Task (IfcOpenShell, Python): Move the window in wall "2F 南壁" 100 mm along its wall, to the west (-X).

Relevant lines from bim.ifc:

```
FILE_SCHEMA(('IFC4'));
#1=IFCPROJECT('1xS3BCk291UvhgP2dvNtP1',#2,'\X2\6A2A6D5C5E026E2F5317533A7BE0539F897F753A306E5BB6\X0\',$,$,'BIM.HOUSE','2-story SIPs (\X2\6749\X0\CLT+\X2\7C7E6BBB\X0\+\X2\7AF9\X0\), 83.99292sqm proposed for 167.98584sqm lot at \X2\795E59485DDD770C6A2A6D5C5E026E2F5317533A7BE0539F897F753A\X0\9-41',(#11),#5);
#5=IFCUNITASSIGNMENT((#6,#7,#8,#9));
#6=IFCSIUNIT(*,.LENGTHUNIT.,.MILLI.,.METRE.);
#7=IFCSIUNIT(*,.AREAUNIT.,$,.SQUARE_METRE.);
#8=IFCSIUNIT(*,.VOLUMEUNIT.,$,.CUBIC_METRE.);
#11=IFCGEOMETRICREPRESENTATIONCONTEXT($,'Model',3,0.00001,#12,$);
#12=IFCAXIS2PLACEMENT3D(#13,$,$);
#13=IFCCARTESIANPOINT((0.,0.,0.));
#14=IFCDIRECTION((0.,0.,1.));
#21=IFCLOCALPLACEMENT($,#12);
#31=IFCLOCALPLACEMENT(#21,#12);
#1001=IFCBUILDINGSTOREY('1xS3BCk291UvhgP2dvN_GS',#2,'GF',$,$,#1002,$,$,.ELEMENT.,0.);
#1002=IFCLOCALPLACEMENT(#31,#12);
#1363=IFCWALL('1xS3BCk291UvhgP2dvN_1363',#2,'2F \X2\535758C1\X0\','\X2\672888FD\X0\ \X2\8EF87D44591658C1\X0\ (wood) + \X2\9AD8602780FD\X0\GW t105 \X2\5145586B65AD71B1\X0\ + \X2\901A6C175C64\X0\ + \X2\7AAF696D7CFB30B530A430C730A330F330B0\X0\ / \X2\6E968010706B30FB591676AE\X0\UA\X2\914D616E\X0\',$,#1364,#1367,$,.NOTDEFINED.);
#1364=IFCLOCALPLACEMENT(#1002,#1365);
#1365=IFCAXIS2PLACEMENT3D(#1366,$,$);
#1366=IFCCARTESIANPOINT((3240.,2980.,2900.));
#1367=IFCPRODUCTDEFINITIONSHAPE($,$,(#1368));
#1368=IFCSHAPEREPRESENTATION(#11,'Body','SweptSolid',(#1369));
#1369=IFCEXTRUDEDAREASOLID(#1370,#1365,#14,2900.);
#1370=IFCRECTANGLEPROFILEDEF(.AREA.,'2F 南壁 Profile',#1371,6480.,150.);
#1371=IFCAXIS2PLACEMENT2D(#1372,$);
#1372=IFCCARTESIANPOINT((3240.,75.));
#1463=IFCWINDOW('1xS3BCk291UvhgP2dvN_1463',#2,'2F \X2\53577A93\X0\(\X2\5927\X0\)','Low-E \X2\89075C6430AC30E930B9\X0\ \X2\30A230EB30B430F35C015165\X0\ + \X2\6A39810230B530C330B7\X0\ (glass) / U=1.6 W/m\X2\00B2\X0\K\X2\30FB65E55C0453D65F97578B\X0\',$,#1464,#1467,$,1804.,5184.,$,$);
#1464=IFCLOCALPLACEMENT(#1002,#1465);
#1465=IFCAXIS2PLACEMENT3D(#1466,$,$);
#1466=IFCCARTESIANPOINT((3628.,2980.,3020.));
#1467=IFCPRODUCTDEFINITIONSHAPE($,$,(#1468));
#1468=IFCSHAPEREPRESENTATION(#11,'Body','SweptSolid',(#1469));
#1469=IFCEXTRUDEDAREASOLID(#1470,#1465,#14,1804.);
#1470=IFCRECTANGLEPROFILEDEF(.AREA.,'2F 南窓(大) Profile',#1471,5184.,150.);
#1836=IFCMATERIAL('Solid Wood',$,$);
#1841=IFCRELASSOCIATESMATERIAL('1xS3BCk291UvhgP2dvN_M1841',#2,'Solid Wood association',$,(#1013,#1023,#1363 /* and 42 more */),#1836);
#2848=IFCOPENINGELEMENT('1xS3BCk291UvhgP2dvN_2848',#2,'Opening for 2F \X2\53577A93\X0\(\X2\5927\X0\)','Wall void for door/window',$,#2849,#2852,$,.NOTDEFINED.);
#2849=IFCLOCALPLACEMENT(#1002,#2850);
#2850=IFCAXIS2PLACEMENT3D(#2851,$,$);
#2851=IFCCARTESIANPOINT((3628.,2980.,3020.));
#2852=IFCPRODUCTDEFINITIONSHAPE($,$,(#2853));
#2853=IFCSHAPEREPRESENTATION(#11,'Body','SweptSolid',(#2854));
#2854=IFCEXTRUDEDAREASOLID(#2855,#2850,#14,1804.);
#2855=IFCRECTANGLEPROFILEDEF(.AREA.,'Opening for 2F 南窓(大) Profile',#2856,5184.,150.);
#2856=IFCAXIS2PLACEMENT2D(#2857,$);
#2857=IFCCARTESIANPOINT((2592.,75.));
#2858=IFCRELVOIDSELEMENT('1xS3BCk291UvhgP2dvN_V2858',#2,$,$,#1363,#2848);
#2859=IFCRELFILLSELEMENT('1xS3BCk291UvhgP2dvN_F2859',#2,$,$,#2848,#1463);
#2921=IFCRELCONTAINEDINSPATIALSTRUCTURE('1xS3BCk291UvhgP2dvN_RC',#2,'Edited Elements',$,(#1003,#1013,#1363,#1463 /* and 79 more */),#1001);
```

```python
import ifcopenshell
import ifcopenshell.api.geometry
import ifcopenshell.util.placement
import ifcopenshell.util.unit

model = ifcopenshell.open("bim.ifc")
unit_scale = ifcopenshell.util.unit.calculate_unit_scale(model)

window = model.by_guid("1xS3BCk291UvhgP2dvN_1463")
opening = window.FillsVoids[0].RelatingOpeningElement
wall = opening.VoidsElements[0].RelatingBuildingElement

wall_matrix = ifcopenshell.util.placement.get_local_placement(wall.ObjectPlacement)
shift = wall_matrix[:3, 0] * -0.1 / unit_scale
before = ifcopenshell.util.placement.get_local_placement(window.ObjectPlacement)[:3, 3].copy()

# The window is not placed relative to its opening, so move both.
for product in (opening, window):
    matrix = ifcopenshell.util.placement.get_local_placement(product.ObjectPlacement)
    matrix[:3, 3] += shift
    ifcopenshell.api.geometry.edit_object_placement(model, product=product, matrix=matrix, is_si=False)

after = ifcopenshell.util.placement.get_local_placement(window.ObjectPlacement)[:3, 3]
print("window moved by", (after - before).round(3) + 0.0)

model.write("bim_v2.ifc")
```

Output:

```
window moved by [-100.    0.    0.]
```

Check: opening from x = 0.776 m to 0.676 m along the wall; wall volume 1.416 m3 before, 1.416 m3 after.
